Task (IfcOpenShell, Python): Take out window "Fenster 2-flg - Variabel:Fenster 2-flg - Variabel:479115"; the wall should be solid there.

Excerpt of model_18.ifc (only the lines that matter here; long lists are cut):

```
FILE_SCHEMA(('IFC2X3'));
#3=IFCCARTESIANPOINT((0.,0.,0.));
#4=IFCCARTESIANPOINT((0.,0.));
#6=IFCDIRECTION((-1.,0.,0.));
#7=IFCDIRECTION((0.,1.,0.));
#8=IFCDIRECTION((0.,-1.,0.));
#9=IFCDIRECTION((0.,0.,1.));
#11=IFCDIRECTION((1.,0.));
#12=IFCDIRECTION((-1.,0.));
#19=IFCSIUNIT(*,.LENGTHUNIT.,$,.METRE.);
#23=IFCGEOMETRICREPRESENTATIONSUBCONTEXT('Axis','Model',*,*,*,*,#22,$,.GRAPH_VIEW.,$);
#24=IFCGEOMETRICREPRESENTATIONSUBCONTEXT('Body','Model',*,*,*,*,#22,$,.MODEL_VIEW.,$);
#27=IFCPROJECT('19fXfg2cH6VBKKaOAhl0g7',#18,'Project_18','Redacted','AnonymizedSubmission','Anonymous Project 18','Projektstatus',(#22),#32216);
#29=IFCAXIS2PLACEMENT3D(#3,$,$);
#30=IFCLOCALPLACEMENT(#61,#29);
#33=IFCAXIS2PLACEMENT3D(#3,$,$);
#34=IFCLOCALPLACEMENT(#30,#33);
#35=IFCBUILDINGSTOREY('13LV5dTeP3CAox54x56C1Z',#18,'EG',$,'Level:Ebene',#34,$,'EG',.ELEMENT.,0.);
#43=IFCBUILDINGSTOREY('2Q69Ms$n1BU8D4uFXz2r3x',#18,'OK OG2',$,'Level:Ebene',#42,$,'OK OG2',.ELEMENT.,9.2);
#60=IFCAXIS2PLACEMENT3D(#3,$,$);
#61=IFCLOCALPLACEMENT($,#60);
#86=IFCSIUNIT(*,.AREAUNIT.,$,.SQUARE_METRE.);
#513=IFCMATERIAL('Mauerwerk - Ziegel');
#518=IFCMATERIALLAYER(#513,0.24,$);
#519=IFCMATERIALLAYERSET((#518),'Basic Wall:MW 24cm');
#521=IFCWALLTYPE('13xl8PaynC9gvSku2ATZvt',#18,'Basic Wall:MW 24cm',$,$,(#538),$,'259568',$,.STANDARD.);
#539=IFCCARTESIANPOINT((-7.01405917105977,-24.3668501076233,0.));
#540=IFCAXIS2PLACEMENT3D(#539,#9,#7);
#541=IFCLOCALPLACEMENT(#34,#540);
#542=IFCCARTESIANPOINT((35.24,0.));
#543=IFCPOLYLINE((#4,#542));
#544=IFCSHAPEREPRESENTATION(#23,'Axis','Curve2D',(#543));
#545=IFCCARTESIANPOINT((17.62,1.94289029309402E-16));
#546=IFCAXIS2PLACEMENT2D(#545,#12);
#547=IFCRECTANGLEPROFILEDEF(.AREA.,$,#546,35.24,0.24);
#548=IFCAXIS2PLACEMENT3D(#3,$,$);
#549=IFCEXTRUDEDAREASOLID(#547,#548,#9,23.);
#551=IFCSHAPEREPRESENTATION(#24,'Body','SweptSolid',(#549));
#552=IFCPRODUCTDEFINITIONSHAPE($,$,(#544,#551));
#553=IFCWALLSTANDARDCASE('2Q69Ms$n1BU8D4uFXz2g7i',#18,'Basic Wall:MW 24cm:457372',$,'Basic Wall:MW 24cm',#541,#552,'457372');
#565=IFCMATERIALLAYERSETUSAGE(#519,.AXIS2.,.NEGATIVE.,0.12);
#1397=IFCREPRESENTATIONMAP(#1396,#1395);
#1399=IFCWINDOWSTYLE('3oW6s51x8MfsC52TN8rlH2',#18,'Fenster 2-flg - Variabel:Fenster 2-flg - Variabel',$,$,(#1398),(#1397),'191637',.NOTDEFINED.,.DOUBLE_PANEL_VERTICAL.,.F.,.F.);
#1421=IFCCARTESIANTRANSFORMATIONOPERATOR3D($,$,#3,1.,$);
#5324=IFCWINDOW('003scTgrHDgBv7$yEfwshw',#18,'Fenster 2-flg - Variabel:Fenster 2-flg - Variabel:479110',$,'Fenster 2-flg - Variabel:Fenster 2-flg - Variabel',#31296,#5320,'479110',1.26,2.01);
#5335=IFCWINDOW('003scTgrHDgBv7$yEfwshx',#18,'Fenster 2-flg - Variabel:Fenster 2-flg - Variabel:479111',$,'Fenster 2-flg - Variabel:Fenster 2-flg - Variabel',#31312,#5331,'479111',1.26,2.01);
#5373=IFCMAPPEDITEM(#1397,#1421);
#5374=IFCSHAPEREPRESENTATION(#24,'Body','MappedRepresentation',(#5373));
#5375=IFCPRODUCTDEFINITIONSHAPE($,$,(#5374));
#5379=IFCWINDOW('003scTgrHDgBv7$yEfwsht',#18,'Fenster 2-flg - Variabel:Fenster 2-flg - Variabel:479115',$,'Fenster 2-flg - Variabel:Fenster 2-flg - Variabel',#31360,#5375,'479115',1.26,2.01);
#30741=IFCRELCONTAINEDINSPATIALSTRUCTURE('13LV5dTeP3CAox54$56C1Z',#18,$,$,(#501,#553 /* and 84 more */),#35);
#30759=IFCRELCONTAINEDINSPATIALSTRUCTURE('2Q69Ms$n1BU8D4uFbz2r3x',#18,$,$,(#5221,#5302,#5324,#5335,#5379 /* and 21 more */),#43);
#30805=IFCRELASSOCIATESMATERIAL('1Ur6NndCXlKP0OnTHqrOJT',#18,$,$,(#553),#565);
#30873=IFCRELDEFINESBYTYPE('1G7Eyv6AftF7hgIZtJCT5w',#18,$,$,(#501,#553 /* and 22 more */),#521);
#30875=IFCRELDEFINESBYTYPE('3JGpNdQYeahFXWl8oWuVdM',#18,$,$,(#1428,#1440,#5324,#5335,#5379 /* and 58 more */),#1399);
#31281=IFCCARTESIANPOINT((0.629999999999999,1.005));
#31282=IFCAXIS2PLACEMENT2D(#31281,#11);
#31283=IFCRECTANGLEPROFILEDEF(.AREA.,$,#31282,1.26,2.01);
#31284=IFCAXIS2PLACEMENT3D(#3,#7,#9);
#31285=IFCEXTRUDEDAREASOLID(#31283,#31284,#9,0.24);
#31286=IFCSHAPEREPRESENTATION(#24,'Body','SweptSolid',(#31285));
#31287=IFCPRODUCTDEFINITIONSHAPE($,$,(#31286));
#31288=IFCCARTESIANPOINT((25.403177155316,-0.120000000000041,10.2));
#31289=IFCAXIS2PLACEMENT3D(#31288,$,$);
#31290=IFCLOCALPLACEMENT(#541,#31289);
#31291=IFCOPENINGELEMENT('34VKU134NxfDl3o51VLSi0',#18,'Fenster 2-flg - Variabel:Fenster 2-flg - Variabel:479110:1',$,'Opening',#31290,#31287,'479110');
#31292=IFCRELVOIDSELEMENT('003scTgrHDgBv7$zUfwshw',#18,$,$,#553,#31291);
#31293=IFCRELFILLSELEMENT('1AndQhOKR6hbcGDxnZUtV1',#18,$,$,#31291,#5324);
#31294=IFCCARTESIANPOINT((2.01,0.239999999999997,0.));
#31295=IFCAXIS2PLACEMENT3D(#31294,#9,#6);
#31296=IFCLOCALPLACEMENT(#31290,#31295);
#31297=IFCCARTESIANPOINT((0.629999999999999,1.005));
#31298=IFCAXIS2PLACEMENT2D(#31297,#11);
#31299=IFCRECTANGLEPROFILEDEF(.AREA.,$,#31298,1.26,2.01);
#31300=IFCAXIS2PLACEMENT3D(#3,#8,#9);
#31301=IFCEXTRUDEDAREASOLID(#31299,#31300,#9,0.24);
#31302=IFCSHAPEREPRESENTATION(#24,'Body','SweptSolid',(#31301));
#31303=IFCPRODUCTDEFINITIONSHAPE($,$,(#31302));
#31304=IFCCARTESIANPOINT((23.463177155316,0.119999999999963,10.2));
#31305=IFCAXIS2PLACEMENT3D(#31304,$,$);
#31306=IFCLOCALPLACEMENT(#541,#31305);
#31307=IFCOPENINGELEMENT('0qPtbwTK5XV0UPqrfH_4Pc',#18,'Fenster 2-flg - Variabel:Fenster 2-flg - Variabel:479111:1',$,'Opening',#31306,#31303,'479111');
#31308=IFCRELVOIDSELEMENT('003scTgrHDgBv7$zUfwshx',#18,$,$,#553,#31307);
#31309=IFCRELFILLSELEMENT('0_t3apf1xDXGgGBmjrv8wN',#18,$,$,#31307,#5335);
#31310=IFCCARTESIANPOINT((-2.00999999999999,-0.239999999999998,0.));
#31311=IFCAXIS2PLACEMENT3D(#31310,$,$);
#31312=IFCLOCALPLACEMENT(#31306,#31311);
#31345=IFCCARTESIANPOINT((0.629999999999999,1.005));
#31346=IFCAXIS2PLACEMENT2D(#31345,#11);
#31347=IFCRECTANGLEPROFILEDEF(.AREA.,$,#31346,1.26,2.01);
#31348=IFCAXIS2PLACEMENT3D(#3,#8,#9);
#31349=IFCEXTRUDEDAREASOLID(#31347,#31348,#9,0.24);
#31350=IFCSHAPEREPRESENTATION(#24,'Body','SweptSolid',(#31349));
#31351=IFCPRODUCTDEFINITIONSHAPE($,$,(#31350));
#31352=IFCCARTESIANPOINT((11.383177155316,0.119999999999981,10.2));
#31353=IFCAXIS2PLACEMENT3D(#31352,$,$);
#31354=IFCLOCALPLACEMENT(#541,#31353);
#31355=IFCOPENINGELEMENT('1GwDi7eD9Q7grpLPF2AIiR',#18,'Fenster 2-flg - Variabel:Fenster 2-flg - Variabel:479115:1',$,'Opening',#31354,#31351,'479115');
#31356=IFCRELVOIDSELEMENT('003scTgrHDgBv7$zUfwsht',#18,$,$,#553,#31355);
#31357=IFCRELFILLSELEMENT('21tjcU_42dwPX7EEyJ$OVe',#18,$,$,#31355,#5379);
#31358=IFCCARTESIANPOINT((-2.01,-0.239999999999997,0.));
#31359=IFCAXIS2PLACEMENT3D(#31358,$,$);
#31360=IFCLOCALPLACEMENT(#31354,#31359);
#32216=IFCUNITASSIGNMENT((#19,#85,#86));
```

```python
import ifcopenshell
import ifcopenshell.api.feature
import ifcopenshell.api.root
import ifcopenshell.geom
import ifcopenshell.util.shape

model = ifcopenshell.open("model_18.ifc")
settings = ifcopenshell.geom.settings()


def volume(element):
    """Net volume in cubic metres, openings subtracted."""
    shape = ifcopenshell.geom.create_shape(settings, element)
    return ifcopenshell.util.shape.get_volume(shape.geometry)


window = model.by_guid("003scTgrHDgBv7$yEfwsht")
opening = window.FillsVoids[0].RelatingOpeningElement
wall = opening.VoidsElements[0].RelatingBuildingElement
before = volume(wall)

ifcopenshell.api.root.remove_product(model, product=window)
ifcopenshell.api.feature.remove_feature(model, feature=opening)

after = volume(wall)

print(f"wall volume {before:.3f} -> {after:.3f} m3")

model.write("model_18_edited.ifc")
```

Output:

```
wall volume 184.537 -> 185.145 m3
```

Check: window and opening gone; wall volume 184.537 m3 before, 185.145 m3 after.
